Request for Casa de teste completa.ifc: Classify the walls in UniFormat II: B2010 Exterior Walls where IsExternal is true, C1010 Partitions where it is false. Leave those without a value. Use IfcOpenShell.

First a look at what the model holds.

```python
import ifcopenshell
import ifcopenshell.util.element

model = ifcopenshell.open("Casa de teste completa.ifc")
print(model.schema)
print("classifications:", [c.Name for c in model.by_type("IfcClassification")])
values = [ifcopenshell.util.element.get_pset(e, "Pset_WallCommon", "IsExternal") for e in model.by_type("IfcWall")]
for value in (True, False, None):
    print("IsExternal", value, values.count(value))
```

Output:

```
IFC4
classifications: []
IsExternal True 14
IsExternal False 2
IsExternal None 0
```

```python
import ifcopenshell
import ifcopenshell.api.classification
import ifcopenshell.util.element

model = ifcopenshell.open("Casa de teste completa.ifc")

system = ifcopenshell.api.classification.add_classification(model, classification="UniFormat II")

walls = model.by_type("IfcWall")
external = {e: ifcopenshell.util.element.get_pset(e, "Pset_WallCommon", "IsExternal") for e in walls}
for flag, code, name in ((True, "B2010", "Exterior Walls"), (False, "C1010", "Partitions")):
    products = [e for e in walls if external[e] is flag]
    ifcopenshell.api.classification.add_reference(
        model, products=products, classification=system, identification=code, name=name
    )
    print(code, len(products))

model.write("Casa de teste completa_v2.ifc")
```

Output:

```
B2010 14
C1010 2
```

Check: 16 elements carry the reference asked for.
